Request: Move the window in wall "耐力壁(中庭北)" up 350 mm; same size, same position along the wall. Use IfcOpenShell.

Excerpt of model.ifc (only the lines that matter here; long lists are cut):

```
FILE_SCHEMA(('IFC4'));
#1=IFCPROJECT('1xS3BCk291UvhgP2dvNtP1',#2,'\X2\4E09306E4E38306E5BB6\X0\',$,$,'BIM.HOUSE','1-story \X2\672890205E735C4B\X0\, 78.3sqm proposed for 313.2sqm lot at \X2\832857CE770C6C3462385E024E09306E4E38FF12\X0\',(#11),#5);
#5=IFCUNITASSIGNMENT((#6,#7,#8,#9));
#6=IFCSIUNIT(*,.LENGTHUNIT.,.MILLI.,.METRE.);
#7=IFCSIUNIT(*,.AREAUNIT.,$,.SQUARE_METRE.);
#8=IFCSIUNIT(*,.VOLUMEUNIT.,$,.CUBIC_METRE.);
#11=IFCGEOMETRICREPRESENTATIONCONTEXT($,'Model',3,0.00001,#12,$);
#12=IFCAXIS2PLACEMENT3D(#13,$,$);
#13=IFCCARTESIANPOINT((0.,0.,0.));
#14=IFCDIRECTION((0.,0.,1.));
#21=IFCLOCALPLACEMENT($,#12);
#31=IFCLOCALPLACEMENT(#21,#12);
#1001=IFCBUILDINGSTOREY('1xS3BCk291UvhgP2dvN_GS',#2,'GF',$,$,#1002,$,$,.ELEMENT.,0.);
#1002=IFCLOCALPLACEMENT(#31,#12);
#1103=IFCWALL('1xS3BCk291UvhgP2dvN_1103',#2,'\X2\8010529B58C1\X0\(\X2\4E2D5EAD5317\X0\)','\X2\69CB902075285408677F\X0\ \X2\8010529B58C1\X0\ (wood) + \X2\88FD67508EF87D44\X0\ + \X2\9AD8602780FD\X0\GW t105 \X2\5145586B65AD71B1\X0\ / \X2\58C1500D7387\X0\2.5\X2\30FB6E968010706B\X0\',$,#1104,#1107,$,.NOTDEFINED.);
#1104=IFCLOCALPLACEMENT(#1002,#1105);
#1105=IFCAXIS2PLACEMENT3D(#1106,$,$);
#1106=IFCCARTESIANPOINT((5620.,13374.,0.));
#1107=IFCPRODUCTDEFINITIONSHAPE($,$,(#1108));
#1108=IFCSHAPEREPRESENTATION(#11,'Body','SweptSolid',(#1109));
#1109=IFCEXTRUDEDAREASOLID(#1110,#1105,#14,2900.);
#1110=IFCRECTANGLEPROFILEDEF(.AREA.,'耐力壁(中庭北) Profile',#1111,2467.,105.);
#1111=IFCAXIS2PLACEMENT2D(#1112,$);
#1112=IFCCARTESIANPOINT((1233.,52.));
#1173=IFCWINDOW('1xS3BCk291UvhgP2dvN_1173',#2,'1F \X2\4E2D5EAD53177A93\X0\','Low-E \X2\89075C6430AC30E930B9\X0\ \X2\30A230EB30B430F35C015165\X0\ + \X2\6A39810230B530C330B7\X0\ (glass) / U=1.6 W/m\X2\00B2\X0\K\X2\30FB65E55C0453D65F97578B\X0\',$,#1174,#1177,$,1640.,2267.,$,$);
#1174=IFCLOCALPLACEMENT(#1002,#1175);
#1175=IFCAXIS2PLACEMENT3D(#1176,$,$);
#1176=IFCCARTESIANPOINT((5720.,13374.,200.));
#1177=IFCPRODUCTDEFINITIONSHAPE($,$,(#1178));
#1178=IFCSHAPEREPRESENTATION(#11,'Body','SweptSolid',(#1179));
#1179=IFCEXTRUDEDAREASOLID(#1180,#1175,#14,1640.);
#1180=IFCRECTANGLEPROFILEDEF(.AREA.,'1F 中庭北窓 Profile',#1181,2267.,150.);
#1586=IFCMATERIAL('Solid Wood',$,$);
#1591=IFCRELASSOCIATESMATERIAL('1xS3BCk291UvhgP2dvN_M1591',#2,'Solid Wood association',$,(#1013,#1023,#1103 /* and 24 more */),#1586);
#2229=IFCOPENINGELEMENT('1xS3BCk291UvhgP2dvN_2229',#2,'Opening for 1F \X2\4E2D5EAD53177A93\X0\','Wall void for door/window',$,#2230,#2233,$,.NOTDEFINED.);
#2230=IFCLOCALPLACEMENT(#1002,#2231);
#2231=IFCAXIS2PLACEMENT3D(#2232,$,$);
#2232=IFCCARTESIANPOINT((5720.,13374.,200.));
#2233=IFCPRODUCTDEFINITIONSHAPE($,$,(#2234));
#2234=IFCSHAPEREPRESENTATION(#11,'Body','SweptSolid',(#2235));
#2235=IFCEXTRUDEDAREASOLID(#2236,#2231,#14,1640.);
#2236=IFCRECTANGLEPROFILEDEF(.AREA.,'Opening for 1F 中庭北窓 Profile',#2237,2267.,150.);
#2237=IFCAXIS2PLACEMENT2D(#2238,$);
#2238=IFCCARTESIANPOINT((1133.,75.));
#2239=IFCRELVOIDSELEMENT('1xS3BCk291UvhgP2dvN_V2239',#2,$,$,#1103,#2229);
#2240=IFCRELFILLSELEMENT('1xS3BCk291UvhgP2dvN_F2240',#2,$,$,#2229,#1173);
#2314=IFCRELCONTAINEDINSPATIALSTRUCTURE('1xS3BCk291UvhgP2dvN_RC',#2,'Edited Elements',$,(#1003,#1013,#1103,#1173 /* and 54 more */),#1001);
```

```python
import numpy as np
import ifcopenshell
import ifcopenshell.api.geometry
import ifcopenshell.util.placement
import ifcopenshell.util.unit

model = ifcopenshell.open("model.ifc")
unit_scale = ifcopenshell.util.unit.calculate_unit_scale(model)

window = model.by_id(1173)
opening = window.FillsVoids[0].RelatingOpeningElement
dz = 0.35 / unit_scale

shift = np.array([0.0, 0.0, dz])
# The window is not placed relative to its opening, so move both.
for product in (opening, window):
    matrix = ifcopenshell.util.placement.get_local_placement(product.ObjectPlacement)
    matrix[:3, 3] += shift
    ifcopenshell.api.geometry.edit_object_placement(model, product=product, matrix=matrix, is_si=False)

print(f"moved by {dz * unit_scale:+.3f} m")

model.write("model-out.ifc")
```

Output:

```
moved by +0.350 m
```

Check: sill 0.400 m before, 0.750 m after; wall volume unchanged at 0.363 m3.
